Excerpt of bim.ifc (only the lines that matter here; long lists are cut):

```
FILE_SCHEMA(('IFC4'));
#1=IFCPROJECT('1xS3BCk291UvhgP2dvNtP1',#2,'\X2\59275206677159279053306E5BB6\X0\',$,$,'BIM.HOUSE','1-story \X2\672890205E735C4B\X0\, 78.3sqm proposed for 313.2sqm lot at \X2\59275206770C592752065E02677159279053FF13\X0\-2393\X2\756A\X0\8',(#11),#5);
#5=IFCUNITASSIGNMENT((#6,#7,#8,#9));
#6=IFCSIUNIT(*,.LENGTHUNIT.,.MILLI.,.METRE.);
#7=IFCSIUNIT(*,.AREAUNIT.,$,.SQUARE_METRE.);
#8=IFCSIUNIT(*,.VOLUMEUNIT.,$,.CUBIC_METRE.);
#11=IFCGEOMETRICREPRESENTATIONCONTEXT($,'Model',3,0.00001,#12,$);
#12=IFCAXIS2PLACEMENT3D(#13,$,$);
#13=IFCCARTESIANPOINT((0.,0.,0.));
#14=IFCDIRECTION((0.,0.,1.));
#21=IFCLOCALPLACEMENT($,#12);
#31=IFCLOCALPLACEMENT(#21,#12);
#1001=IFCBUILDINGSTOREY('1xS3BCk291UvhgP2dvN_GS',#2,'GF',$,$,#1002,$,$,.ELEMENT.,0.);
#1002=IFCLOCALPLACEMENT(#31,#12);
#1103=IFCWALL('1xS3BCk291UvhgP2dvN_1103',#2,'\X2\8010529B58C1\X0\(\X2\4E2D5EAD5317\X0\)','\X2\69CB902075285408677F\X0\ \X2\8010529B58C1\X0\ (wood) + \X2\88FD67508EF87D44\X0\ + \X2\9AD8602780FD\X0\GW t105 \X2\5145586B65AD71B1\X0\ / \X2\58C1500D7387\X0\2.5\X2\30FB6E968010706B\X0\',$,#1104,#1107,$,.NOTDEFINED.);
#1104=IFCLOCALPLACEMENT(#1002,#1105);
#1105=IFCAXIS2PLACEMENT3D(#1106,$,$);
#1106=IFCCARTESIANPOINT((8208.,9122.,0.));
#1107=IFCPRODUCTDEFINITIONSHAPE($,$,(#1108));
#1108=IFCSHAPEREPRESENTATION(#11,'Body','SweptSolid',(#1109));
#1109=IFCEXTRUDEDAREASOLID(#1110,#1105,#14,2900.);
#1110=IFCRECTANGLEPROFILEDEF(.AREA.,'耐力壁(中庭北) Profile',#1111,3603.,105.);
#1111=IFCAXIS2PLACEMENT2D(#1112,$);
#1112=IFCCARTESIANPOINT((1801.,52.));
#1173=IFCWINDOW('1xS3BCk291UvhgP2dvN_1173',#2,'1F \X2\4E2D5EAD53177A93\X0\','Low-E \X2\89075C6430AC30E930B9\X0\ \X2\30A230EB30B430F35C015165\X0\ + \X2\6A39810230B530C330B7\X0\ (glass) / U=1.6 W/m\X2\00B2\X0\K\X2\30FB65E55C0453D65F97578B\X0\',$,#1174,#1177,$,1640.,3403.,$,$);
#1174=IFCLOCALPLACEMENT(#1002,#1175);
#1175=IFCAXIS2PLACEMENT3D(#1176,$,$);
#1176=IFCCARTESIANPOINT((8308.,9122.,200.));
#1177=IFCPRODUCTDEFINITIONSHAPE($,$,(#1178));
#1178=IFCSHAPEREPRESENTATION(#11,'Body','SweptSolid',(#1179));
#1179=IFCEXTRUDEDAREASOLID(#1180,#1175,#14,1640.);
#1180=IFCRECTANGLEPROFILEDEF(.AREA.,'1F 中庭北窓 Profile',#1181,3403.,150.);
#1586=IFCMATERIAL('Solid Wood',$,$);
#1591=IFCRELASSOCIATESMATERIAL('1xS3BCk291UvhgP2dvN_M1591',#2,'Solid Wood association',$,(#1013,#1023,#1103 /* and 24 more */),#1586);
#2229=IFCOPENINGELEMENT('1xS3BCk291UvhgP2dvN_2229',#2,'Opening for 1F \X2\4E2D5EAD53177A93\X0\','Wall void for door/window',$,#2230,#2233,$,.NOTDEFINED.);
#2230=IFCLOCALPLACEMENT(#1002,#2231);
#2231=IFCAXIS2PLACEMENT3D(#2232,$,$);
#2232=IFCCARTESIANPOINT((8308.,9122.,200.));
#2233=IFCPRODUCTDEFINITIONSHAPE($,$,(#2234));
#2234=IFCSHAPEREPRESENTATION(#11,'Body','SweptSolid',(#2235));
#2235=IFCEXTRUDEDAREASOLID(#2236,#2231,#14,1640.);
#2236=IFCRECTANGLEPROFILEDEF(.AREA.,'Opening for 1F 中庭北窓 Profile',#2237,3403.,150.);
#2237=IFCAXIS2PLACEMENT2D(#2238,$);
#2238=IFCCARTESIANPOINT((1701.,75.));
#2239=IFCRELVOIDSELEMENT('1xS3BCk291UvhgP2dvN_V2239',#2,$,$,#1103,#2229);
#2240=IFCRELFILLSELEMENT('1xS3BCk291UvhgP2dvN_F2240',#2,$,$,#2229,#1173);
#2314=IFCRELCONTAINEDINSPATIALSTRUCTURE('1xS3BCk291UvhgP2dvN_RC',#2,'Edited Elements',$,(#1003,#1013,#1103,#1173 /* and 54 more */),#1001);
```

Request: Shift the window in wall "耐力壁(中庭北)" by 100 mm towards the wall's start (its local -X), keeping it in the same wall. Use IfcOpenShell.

```python
import ifcopenshell
import ifcopenshell.api.geometry
import ifcopenshell.util.placement

model = ifcopenshell.open("bim.ifc")

window = model.by_id(1173)
opening = window.FillsVoids[0].RelatingOpeningElement
wall = opening.VoidsElements[0].RelatingBuildingElement

wall_matrix = ifcopenshell.util.placement.get_local_placement(wall.ObjectPlacement)
shift = wall_matrix[:3, 0] * -100.0
before = ifcopenshell.util.placement.get_local_placement(window.ObjectPlacement)[:3, 3].copy()

# The window is not placed relative to its opening, so move both.
for product in (opening, window):
    matrix = ifcopenshell.util.placement.get_local_placement(product.ObjectPlacement)
    matrix[:3, 3] += shift
    ifcopenshell.api.geometry.edit_object_placement(model, product=product, matrix=matrix, is_si=False)

after = ifcopenshell.util.placement.get_local_placement(window.ObjectPlacement)[:3, 3]
print("window moved by", (after - before).round(3) + 0.0)

model.write("bim_updated.ifc")
```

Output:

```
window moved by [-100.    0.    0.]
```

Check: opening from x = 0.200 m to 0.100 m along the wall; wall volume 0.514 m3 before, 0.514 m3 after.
